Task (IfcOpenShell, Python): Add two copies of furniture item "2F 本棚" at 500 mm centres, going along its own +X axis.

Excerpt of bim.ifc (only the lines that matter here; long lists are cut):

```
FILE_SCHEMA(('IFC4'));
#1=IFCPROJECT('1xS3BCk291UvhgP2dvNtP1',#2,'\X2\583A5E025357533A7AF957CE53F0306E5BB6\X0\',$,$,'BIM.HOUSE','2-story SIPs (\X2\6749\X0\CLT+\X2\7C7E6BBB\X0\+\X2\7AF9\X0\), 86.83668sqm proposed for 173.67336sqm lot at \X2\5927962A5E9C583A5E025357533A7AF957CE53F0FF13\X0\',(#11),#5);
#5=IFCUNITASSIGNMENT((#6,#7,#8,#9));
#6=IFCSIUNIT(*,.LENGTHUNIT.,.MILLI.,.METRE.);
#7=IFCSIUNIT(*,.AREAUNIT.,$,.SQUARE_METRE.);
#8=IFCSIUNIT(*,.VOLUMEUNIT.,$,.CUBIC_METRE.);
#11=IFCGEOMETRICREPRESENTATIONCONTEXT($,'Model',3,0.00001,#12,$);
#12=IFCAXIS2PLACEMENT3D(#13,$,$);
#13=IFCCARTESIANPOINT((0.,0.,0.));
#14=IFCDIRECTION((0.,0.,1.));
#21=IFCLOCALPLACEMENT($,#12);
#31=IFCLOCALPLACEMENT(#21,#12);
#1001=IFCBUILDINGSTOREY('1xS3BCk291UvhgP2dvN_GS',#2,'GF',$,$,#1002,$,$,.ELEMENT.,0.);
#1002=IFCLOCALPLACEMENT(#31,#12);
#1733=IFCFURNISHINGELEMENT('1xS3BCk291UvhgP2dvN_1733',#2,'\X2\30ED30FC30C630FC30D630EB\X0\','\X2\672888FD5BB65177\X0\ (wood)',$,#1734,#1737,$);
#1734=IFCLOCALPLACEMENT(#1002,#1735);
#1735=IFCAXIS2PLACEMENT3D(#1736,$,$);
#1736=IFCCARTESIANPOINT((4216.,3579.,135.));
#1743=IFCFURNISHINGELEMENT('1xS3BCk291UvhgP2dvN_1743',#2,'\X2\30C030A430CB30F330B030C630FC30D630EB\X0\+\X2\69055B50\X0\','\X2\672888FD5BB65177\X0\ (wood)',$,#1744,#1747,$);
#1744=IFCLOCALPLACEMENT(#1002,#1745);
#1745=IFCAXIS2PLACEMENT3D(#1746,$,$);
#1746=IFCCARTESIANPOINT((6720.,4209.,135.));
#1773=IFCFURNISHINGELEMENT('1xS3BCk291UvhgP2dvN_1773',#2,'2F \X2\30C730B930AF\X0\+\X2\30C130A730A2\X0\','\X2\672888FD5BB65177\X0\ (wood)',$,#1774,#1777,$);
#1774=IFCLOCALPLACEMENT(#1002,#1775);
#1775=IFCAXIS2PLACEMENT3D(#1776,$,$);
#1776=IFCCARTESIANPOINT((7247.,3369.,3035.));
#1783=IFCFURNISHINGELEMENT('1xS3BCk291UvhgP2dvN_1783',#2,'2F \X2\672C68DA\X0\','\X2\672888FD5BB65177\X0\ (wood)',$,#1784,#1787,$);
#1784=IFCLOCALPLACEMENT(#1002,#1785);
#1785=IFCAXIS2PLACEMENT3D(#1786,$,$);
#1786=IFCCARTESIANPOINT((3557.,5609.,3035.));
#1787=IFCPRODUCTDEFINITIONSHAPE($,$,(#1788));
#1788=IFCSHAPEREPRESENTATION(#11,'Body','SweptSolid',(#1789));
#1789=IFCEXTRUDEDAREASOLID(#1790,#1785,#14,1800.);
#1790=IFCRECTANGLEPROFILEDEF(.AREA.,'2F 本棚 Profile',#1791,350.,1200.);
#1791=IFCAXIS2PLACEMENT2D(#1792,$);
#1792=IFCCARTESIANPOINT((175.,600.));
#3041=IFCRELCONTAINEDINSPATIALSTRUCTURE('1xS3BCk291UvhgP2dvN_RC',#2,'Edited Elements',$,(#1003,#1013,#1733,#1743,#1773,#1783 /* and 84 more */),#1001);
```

```python
import ifcopenshell
import ifcopenshell.api.geometry
import ifcopenshell.api.root
import ifcopenshell.util.element
import ifcopenshell.util.placement

model = ifcopenshell.open("bim.ifc")


def reuse_history(source, copy):
    """copy_class also copies each property set's owner history, people and application; keep the originals."""
    for rel in copy.IsDefinedBy:
        if rel.is_a("IfcRelDefinesByProperties") and (history := rel.RelatingPropertyDefinition.OwnerHistory):
            rel.RelatingPropertyDefinition.OwnerHistory = source.OwnerHistory
            ifcopenshell.util.element.remove_deep2(model, history)


source = model.by_guid("1xS3BCk291UvhgP2dvN_1783")
base = ifcopenshell.util.placement.get_local_placement(source.ObjectPlacement)
step = base[:3, 0] * 500.0

for i in range(1, 3):
    copy = ifcopenshell.api.root.copy_class(model, product=source)
    copy.Representation = ifcopenshell.util.element.copy_deep(
        model, source.Representation, exclude=["IfcGeometricRepresentationContext", "IfcRepresentationMap"]
    )
    reuse_history(source, copy)
    matrix = base.copy()
    matrix[:3, 3] += i * step
    print("added at", matrix[:3, 3].round(3) + 0.0)
    ifcopenshell.api.geometry.edit_object_placement(model, product=copy, matrix=matrix, is_si=False)

model.write("bim_edited.ifc")
```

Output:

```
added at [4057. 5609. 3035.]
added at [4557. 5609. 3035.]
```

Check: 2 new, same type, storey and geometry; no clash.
